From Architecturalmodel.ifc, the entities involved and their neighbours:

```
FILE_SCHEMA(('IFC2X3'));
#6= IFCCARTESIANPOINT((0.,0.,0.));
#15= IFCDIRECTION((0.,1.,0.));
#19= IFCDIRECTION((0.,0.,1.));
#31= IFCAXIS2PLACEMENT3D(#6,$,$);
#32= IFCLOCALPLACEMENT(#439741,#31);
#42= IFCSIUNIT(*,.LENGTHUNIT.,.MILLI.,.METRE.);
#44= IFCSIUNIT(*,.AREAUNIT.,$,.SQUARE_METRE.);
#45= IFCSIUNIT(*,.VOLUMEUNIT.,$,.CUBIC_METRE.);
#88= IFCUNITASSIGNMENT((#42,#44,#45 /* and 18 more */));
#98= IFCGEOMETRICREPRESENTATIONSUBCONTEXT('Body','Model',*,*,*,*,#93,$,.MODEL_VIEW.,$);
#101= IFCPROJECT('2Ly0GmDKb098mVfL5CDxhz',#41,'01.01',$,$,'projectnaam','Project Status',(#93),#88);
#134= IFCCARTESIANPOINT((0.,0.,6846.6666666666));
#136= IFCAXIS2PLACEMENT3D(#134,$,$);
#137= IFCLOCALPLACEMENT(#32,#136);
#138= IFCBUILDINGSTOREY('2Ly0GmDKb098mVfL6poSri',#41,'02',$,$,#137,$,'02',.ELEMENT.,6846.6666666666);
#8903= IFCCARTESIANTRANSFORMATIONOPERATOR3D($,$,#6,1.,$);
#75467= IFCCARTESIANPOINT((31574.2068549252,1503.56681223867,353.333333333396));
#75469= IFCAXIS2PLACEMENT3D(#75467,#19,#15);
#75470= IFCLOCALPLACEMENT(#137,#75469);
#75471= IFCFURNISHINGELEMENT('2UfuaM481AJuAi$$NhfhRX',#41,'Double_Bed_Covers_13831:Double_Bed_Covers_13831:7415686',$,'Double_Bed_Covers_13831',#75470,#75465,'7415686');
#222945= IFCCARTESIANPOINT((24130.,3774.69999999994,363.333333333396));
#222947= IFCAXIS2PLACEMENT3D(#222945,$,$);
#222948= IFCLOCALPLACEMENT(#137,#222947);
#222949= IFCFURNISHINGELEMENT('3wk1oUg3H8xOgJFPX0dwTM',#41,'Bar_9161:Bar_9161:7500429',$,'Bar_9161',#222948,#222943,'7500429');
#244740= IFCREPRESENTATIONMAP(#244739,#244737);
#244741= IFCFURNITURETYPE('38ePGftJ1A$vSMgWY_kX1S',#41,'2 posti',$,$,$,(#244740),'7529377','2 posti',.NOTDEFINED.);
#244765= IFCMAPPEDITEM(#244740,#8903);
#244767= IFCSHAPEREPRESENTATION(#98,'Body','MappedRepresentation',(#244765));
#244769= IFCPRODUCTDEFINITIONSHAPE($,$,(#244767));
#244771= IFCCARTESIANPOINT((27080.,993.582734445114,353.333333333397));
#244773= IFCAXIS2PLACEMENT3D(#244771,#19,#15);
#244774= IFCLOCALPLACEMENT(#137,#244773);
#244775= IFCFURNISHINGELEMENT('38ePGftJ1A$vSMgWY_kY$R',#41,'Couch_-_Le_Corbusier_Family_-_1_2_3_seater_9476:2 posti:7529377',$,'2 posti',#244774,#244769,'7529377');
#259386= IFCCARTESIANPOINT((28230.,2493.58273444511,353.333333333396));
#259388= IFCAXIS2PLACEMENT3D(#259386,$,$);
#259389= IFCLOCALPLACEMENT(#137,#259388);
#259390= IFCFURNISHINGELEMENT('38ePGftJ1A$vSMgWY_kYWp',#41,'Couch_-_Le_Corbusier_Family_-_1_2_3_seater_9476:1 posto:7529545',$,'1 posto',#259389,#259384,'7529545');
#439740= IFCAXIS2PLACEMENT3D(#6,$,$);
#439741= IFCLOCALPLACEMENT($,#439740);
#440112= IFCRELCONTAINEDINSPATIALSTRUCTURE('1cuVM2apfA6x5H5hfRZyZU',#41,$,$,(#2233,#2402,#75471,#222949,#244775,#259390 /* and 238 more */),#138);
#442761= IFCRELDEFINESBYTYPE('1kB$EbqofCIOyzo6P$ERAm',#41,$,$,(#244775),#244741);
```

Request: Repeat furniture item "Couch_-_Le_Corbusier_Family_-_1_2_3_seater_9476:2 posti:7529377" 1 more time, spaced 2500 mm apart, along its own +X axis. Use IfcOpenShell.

```python
import ifcopenshell
import ifcopenshell.api.geometry
import ifcopenshell.api.root
import ifcopenshell.util.element
import ifcopenshell.util.placement

model = ifcopenshell.open("Architecturalmodel.ifc")

source = model.by_id(244775)
base = ifcopenshell.util.placement.get_local_placement(source.ObjectPlacement)
step = base[:3, 0] * 2500.0

for i in range(1, 2):
    copy = ifcopenshell.api.root.copy_class(model, product=source)
    copy.Representation = ifcopenshell.util.element.copy_deep(
        model, source.Representation, exclude=["IfcGeometricRepresentationContext", "IfcRepresentationMap"]
    )
    copy.Name = "Couch_-_Le_Corbusier_Family_-_1_2_3_seater_9476:2 posti"
    copy.Tag = None
    matrix = base.copy()
    matrix[:3, 3] += i * step
    print("added at", matrix[:3, 3].round(3) + 0.0)
    ifcopenshell.api.geometry.edit_object_placement(model, product=copy, matrix=matrix, is_si=False)

model.write("Architecturalmodel-out.ifc")
```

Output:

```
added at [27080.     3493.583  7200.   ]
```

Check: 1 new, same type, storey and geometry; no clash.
